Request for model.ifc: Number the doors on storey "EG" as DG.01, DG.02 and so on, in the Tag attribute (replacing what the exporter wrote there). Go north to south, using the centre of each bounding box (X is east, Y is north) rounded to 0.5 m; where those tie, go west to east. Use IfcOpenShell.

First a look at what the model holds.

```python
import ifcopenshell
import ifcopenshell.util.element
import ifcopenshell.util.placement

model = ifcopenshell.open("model.ifc")
print(model.schema)
storey = next(s for s in model.by_type("IfcBuildingStorey") if s.Name == "EG")
doors = [e for e in ifcopenshell.util.element.get_decomposition(storey) if e.is_a("IfcDoor")]
for e in sorted(doors, key=lambda e: e.id()):
    origin = ifcopenshell.util.placement.get_local_placement(e.ObjectPlacement)[:3, 3]
    print(e.id(), e.Tag, e.Name, origin.round(2) + 0.0, sep=" | ")
```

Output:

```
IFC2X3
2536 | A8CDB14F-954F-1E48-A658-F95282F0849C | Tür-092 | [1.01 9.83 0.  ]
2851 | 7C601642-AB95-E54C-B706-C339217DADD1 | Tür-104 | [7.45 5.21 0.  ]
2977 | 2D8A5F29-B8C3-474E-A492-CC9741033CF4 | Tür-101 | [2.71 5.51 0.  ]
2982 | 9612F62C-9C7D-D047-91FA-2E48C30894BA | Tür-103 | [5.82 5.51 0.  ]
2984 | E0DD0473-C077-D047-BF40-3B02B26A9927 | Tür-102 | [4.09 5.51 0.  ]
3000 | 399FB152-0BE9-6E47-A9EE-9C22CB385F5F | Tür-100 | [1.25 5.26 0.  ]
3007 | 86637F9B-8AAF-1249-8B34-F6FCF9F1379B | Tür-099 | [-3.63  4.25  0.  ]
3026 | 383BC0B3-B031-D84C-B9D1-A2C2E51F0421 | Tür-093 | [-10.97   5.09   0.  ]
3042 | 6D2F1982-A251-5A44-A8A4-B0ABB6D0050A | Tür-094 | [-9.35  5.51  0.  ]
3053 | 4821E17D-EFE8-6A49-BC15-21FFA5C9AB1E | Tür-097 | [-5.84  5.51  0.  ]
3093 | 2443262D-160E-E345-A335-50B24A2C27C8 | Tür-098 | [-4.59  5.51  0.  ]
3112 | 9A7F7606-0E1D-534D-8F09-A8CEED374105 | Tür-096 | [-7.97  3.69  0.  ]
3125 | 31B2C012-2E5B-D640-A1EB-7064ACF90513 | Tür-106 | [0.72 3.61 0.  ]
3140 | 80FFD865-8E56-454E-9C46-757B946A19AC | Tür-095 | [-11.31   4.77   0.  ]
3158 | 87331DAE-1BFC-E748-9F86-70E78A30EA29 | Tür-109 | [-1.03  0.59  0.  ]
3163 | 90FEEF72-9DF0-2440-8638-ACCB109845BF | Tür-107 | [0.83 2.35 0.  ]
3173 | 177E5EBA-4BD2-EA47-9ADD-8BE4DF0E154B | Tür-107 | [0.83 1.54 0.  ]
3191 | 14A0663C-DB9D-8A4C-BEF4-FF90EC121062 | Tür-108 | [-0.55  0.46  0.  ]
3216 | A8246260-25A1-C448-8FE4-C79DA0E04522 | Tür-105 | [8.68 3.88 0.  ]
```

```python
import ifcopenshell
import ifcopenshell.geom
import ifcopenshell.util.element
import ifcopenshell.util.shape

model = ifcopenshell.open("model.ifc")
settings = ifcopenshell.geom.settings()
settings.set("use-world-coords", True)


def centre(element):
    shape = ifcopenshell.geom.create_shape(settings, element)
    return ifcopenshell.util.shape.get_bbox_centroid(shape.geometry)


storey = next(s for s in model.by_type("IfcBuildingStorey") if s.Name == "EG")
doors = [e for e in ifcopenshell.util.element.get_decomposition(storey) if e.is_a("IfcDoor")]

# Insertion points can sit at a corner or the storey origin, so sort by the geometry (in metres).
centres = {e: centre(e) for e in doors}
doors.sort(key=lambda e: (-round(centres[e][1] / 0.5), centres[e][0]))

for i, e in enumerate(doors, start=1):
    number = f"DG.{i:02d}"
    e.Tag = number
    print(e.id(), number)

model.write("model_v2.ifc")
```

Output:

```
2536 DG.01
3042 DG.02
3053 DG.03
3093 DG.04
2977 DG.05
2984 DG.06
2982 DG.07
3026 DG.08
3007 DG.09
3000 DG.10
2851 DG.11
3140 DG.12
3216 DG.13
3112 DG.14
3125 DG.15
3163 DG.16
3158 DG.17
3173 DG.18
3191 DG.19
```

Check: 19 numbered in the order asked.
